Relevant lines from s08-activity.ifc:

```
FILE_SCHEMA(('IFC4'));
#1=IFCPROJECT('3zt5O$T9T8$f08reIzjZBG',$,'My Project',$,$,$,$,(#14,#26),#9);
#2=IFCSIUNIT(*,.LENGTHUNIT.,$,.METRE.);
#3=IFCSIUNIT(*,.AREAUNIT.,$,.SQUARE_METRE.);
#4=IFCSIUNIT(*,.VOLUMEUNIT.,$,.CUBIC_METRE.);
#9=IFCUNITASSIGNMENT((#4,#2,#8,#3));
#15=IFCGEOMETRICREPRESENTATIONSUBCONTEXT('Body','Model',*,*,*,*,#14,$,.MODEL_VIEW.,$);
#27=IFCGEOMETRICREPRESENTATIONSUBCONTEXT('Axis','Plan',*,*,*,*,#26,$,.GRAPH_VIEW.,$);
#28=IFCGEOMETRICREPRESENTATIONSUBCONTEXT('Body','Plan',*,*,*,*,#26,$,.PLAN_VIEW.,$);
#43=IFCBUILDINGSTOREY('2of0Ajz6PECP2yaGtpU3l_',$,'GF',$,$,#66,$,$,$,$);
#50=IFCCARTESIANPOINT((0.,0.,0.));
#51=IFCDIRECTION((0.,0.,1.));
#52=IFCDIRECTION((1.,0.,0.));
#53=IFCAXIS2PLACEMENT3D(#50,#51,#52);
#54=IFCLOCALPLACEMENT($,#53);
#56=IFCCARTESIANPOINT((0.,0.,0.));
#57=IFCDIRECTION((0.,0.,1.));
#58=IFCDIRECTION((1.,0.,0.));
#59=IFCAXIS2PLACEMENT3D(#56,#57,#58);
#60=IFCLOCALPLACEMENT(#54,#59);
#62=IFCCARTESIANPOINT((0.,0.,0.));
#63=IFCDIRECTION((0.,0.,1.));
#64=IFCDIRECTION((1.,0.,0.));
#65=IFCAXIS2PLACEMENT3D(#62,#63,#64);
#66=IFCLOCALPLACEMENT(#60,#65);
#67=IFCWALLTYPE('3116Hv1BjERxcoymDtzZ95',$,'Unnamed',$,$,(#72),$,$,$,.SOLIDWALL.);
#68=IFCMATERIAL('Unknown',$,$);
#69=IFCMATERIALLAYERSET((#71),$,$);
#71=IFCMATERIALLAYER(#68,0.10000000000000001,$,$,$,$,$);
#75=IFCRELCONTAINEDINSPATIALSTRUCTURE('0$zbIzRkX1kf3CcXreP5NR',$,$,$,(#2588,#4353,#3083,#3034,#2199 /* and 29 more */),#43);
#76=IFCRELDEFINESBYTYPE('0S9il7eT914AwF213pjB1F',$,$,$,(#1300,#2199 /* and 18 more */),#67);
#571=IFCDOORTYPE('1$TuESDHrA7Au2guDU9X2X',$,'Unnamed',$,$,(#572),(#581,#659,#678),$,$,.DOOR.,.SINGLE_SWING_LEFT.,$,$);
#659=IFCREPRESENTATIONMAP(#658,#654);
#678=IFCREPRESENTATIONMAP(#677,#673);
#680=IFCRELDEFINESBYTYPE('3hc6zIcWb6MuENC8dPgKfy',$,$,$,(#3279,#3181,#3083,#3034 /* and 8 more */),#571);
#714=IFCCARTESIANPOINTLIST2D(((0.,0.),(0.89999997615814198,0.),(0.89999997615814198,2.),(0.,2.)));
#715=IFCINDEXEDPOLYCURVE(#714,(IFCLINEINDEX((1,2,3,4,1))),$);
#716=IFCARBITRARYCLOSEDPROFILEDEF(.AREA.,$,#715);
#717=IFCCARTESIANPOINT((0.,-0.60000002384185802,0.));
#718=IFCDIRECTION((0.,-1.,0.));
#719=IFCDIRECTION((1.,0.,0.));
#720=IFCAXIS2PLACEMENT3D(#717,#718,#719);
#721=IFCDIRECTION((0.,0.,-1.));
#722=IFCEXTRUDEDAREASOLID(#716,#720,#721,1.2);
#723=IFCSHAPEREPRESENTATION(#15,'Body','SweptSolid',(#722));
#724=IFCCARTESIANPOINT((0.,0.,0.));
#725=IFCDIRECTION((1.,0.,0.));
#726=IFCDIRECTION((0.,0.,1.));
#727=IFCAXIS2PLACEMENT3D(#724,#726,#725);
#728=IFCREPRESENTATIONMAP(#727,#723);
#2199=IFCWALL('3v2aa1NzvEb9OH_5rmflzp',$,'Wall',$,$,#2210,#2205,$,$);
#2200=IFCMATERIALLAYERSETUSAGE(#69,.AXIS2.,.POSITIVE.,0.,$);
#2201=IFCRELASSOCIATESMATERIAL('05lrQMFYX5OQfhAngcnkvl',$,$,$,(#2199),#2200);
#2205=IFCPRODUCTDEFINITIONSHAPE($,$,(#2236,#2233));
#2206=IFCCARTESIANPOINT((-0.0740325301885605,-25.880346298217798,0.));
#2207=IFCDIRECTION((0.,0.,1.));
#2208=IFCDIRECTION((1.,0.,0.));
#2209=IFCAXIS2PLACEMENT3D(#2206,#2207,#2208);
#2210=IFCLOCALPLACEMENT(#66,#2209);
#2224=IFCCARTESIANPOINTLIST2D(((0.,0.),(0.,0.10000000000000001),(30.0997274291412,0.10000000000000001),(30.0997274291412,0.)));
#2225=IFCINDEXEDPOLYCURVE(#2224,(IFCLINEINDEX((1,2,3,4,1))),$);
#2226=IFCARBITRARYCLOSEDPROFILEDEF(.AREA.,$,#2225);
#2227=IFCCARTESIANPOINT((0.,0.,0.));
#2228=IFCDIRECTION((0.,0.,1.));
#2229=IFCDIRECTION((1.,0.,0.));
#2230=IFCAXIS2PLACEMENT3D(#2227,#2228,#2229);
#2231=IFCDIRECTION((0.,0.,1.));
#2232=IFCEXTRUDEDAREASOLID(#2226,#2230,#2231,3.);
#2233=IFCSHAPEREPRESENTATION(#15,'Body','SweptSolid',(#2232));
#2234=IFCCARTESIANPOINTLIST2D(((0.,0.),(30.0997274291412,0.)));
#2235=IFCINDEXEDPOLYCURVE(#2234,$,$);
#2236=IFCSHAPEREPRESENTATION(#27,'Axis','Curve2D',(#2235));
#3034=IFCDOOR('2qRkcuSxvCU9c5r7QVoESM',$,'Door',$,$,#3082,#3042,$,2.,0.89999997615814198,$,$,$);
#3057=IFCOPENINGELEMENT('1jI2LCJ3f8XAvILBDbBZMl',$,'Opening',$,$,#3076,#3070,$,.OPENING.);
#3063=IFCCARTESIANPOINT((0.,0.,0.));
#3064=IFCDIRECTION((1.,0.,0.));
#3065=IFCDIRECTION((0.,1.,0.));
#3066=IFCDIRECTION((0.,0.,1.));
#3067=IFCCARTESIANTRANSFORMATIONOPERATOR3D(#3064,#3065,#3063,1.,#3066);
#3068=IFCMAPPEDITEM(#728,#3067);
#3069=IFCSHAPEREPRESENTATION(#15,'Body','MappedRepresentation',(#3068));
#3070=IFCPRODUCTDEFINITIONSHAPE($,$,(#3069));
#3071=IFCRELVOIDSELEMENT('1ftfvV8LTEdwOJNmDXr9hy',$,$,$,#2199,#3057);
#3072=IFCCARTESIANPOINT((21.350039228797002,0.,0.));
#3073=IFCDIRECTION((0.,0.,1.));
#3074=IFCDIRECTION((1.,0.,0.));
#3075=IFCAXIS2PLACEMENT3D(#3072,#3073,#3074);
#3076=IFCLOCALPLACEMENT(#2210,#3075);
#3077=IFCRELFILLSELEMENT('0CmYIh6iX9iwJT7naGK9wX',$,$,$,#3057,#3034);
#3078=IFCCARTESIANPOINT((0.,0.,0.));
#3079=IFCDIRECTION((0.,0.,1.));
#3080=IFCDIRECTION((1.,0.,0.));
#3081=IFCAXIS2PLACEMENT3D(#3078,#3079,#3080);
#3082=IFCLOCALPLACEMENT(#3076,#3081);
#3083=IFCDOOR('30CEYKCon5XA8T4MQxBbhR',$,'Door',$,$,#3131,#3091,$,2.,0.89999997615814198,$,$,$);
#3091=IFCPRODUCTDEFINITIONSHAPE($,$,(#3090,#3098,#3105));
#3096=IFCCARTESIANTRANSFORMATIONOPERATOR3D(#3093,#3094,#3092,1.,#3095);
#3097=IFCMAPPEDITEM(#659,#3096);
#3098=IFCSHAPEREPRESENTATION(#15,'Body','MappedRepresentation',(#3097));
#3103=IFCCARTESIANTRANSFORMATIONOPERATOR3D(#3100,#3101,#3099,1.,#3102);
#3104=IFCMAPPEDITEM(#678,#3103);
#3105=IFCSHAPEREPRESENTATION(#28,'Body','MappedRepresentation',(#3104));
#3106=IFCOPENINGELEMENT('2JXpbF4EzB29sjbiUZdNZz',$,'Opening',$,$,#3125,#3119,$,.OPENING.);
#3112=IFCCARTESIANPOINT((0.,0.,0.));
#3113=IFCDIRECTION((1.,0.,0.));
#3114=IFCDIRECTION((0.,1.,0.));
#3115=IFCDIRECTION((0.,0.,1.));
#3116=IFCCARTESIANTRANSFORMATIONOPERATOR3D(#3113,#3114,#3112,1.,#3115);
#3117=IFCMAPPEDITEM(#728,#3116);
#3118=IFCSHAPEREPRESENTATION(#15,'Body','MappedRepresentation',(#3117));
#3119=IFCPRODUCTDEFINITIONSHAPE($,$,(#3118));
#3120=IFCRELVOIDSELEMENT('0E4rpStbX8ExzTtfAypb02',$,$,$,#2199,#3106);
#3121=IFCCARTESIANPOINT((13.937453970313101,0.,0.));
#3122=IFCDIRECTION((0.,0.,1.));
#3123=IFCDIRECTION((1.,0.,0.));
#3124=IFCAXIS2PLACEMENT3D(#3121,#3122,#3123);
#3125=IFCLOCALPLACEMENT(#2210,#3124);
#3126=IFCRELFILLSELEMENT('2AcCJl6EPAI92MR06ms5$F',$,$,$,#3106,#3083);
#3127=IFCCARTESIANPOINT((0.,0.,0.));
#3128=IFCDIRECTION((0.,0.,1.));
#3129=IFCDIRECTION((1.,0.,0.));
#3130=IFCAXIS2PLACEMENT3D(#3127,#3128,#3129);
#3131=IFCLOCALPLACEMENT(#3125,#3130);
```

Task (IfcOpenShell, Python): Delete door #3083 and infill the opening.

```python
import ifcopenshell
import ifcopenshell.api.feature
import ifcopenshell.api.root
import ifcopenshell.geom
import ifcopenshell.util.shape

model = ifcopenshell.open("s08-activity.ifc")
settings = ifcopenshell.geom.settings()


def volume(element):
    """Net volume in cubic metres, openings subtracted."""
    shape = ifcopenshell.geom.create_shape(settings, element)
    return ifcopenshell.util.shape.get_volume(shape.geometry)


door = model.by_guid("30CEYKCon5XA8T4MQxBbhR")
opening = door.FillsVoids[0].RelatingOpeningElement
wall = opening.VoidsElements[0].RelatingBuildingElement
before = volume(wall)

ifcopenshell.api.root.remove_product(model, product=door)
ifcopenshell.api.feature.remove_feature(model, feature=opening)

after = volume(wall)

print(f"wall volume {before:.3f} -> {after:.3f} m3")

model.write("s08-activity_updated.ifc")
```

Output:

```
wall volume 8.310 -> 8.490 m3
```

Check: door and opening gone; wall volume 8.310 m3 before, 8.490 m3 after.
